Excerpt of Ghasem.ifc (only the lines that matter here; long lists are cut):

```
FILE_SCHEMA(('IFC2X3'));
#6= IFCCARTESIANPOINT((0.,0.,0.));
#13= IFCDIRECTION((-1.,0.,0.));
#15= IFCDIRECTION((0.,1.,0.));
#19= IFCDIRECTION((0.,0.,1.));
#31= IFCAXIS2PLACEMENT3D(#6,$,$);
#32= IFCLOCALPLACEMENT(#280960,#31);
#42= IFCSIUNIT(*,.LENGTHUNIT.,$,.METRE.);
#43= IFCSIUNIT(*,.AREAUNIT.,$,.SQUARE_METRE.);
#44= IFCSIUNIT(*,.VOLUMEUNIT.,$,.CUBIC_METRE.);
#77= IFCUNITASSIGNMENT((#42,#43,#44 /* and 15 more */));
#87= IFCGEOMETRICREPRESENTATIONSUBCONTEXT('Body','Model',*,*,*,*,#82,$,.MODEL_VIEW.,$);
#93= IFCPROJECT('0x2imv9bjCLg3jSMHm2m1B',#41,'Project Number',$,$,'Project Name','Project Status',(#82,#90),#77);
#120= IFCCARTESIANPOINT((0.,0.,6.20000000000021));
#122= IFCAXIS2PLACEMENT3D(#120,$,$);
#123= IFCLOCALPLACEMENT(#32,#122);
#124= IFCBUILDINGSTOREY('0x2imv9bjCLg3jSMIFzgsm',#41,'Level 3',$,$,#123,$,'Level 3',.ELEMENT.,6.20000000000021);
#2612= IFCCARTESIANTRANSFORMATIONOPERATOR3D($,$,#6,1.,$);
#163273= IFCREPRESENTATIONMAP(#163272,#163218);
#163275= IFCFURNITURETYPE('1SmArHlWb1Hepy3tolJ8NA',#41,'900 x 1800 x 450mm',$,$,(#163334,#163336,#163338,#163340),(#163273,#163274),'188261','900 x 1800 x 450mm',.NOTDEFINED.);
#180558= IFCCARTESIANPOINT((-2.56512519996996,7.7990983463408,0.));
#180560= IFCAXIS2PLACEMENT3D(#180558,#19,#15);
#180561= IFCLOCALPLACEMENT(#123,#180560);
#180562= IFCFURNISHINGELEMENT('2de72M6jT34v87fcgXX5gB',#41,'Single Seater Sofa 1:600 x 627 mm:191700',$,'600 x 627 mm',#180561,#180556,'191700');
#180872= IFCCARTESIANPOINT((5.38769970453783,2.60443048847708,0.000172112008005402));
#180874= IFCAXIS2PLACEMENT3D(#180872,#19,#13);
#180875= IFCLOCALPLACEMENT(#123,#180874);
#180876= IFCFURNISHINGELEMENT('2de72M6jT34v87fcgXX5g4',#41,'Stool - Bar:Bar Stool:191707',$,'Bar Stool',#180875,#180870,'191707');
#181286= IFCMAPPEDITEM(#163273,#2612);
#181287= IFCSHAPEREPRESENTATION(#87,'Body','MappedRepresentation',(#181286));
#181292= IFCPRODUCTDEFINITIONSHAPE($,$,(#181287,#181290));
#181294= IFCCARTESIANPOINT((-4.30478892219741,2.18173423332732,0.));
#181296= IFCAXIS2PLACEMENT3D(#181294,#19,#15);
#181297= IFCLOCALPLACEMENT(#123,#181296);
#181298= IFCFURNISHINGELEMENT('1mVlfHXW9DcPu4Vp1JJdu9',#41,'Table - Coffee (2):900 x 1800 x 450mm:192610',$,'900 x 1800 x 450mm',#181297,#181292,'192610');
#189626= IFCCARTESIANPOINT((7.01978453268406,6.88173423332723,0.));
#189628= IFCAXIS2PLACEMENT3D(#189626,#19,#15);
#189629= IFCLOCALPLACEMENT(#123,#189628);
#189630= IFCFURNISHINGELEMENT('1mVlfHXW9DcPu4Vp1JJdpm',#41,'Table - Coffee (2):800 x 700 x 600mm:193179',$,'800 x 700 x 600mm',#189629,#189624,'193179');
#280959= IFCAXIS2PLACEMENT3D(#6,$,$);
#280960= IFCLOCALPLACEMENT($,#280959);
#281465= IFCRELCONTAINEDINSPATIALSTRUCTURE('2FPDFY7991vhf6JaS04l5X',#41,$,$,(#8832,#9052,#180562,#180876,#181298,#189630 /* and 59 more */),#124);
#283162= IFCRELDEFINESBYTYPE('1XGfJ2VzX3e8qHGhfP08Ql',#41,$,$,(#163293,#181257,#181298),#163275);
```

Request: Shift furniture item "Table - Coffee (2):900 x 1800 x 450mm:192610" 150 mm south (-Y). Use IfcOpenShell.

```python
import ifcopenshell
import ifcopenshell.api.geometry
import ifcopenshell.util.placement

model = ifcopenshell.open("Ghasem.ifc")

item = model.by_id(181298)
matrix = ifcopenshell.util.placement.get_local_placement(item.ObjectPlacement)
matrix[1, 3] -= 0.15
ifcopenshell.api.geometry.edit_object_placement(model, product=item, matrix=matrix, is_si=False)

print(ifcopenshell.util.placement.get_local_placement(item.ObjectPlacement).round(3) + 0.0)

model.write("Ghasem_edited.ifc")
```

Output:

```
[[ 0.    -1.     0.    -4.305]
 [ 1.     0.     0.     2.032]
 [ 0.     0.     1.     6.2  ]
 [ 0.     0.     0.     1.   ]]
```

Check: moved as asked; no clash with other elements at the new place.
